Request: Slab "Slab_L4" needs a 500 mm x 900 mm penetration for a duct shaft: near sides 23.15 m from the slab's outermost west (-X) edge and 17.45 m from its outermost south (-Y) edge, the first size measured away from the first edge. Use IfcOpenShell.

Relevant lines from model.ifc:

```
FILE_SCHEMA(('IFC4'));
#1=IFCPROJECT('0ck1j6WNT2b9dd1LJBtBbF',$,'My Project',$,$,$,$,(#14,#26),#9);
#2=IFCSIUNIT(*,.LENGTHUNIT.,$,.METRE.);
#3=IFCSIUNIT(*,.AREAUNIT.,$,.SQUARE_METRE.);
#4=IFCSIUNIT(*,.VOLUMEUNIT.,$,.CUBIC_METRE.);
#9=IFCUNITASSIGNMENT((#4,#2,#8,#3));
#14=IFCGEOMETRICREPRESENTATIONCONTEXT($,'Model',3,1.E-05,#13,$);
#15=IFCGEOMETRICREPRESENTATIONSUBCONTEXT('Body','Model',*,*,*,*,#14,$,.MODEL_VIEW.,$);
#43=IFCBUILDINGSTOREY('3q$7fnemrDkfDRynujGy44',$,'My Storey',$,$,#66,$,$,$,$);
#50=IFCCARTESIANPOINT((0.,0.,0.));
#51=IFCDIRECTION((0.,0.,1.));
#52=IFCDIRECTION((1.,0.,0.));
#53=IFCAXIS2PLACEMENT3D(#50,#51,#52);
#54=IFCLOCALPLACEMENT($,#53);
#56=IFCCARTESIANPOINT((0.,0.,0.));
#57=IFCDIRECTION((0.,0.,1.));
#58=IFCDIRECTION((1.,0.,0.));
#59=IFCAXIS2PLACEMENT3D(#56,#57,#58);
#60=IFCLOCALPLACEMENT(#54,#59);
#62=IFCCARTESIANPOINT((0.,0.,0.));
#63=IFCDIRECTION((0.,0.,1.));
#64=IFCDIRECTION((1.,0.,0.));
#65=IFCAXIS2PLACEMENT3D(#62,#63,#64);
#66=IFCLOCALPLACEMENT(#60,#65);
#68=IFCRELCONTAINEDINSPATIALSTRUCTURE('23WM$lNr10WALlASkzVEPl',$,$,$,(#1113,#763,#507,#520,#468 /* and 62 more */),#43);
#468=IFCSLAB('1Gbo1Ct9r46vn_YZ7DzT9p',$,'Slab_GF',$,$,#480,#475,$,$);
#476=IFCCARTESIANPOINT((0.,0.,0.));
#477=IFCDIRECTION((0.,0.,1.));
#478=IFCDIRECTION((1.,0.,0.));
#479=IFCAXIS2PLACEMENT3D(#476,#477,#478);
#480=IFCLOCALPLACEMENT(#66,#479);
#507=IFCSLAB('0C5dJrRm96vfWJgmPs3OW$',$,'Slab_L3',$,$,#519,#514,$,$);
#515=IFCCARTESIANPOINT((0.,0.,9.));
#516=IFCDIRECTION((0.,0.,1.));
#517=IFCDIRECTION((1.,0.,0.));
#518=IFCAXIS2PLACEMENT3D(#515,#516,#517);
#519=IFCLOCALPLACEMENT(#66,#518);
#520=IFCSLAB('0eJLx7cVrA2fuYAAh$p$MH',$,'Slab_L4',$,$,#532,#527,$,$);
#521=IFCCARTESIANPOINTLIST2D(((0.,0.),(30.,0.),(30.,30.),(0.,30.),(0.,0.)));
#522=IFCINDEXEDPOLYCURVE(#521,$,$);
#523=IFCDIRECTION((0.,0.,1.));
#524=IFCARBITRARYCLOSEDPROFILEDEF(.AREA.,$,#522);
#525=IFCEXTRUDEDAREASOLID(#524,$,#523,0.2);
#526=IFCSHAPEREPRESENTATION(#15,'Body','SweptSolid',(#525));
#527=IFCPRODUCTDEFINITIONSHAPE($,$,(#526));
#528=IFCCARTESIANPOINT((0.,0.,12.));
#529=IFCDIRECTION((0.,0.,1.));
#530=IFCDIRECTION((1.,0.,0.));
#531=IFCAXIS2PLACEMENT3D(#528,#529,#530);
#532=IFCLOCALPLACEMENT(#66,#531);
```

```python
import numpy as np
import ifcopenshell
import ifcopenshell.api.feature
import ifcopenshell.api.geometry
import ifcopenshell.api.root
import ifcopenshell.geom
import ifcopenshell.util.placement
import ifcopenshell.util.representation
import ifcopenshell.util.shape
import ifcopenshell.util.unit

model = ifcopenshell.open("model.ifc")
unit_scale = ifcopenshell.util.unit.calculate_unit_scale(model)
settings = ifcopenshell.geom.settings()


def volume(element):
    """Net volume in cubic metres, openings subtracted."""
    shape = ifcopenshell.geom.create_shape(settings, element)
    return ifcopenshell.util.shape.get_volume(shape.geometry)


slab = model.by_id(520)
before = volume(slab)

# Extent in the slab's own axes, in metres. The edges named are its -X and -Y sides.
slab_shape = ifcopenshell.geom.create_shape(settings, slab)
vertices = ifcopenshell.util.shape.get_vertices(slab_shape.geometry)
x_min, y_min, bottom = vertices.min(axis=0)
top = vertices[:, 2].max()

opening = ifcopenshell.api.root.create_entity(model, ifc_class="IfcOpeningElement", name="Duct shaft opening", predefined_type="OPENING")
context = ifcopenshell.util.representation.get_context(model, "Model", "Body", "MODEL_VIEW")
width, depth = 0.5, 0.9
outline = [(0.0, 0.0), (width, 0.0), (width, depth), (0.0, depth), (0.0, 0.0)]
# Overshoot both faces by 50 mm so the cut is clean.
shape = ifcopenshell.api.geometry.add_slab_representation(
    model, context=context, depth=top - bottom + 0.1, polyline=outline
)
ifcopenshell.api.geometry.assign_representation(model, product=opening, representation=shape)

matrix = ifcopenshell.util.placement.get_local_placement(slab.ObjectPlacement)
matrix[:, 3] = matrix @ np.append(np.array([x_min + 23.15, y_min + 17.45, bottom - 0.05]) / unit_scale, 1.0)
ifcopenshell.api.geometry.edit_object_placement(model, product=opening, matrix=matrix, is_si=False)
ifcopenshell.api.feature.add_feature(model, feature=opening, element=slab)

after = volume(slab)

print(f"slab volume {before:.3f} -> {after:.3f} m3")

model.write("model-out.ifc")
```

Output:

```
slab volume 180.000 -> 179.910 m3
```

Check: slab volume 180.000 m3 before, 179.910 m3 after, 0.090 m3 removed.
